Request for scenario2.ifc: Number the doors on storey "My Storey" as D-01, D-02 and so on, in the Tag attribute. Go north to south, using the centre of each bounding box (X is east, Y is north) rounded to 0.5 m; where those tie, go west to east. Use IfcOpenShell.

First a look at what the model holds.

```python
import ifcopenshell
import ifcopenshell.util.element
import ifcopenshell.util.placement

model = ifcopenshell.open("scenario2.ifc")
print(model.schema)
storey = next(s for s in model.by_type("IfcBuildingStorey") if s.Name == "My Storey")
doors = [e for e in ifcopenshell.util.element.get_decomposition(storey) if e.is_a("IfcDoor")]
for e in sorted(doors, key=lambda e: e.id()):
    origin = ifcopenshell.util.placement.get_local_placement(e.ObjectPlacement)[:3, 3]
    print(e.id(), e.Tag, e.Name, origin.round(2) + 0.0, sep=" | ")
```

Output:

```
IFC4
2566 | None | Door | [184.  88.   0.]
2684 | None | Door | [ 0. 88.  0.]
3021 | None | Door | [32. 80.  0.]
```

```python
import ifcopenshell
import ifcopenshell.geom
import ifcopenshell.util.element
import ifcopenshell.util.shape

model = ifcopenshell.open("scenario2.ifc")
settings = ifcopenshell.geom.settings()
settings.set("use-world-coords", True)


def centre(element):
    shape = ifcopenshell.geom.create_shape(settings, element)
    return ifcopenshell.util.shape.get_bbox_centroid(shape.geometry)


storey = next(s for s in model.by_type("IfcBuildingStorey") if s.Name == "My Storey")
doors = [e for e in ifcopenshell.util.element.get_decomposition(storey) if e.is_a("IfcDoor")]

# Insertion points can sit at a corner or the storey origin, so sort by the geometry (in metres).
centres = {e: centre(e) for e in doors}
doors.sort(key=lambda e: (-round(centres[e][1] / 0.5), centres[e][0]))

for i, e in enumerate(doors, start=1):
    number = f"D-{i:02d}"
    e.Tag = number
    print(e.id(), number)

model.write("scenario2-out.ifc")
```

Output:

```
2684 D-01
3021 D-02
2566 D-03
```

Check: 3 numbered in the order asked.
